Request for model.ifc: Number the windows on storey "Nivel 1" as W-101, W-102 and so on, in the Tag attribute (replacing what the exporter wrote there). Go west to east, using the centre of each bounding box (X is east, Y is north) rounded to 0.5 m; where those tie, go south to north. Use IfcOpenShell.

First a look at what the model holds.

```python
import ifcopenshell
import ifcopenshell.util.element
import ifcopenshell.util.placement

model = ifcopenshell.open("model.ifc")
print(model.schema)
storey = next(s for s in model.by_type("IfcBuildingStorey") if s.Name == "Nivel 1")
windows = [e for e in ifcopenshell.util.element.get_decomposition(storey) if e.is_a("IfcWindow")]
for e in sorted(windows, key=lambda e: e.id()):
    origin = ifcopenshell.util.placement.get_local_placement(e.ObjectPlacement)[:3, 3]
    print(e.id(), e.Tag, e.Name, origin.round(2) + 0.0, sep=" | ")
```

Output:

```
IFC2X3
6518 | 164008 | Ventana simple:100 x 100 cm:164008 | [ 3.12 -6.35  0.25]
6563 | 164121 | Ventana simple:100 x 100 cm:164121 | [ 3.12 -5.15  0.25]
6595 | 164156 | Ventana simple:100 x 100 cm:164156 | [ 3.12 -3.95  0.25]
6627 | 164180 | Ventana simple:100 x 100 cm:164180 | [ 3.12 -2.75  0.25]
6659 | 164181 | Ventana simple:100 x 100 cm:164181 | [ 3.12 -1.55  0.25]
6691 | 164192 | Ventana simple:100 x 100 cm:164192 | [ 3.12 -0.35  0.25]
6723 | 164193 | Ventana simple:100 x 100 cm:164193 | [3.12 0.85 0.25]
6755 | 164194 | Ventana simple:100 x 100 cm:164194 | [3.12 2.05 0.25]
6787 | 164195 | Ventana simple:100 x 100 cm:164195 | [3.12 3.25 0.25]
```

```python
import ifcopenshell
import ifcopenshell.geom
import ifcopenshell.util.element
import ifcopenshell.util.shape

model = ifcopenshell.open("model.ifc")
settings = ifcopenshell.geom.settings()
settings.set("use-world-coords", True)


def centre(element):
    shape = ifcopenshell.geom.create_shape(settings, element)
    return ifcopenshell.util.shape.get_bbox_centroid(shape.geometry)


storey = next(s for s in model.by_type("IfcBuildingStorey") if s.Name == "Nivel 1")
windows = [e for e in ifcopenshell.util.element.get_decomposition(storey) if e.is_a("IfcWindow")]

# Insertion points can sit at a corner or the storey origin, so sort by the geometry (in metres).
centres = {e: centre(e) for e in windows}
windows.sort(key=lambda e: (round(centres[e][0] / 0.5), centres[e][1]))

for i, e in enumerate(windows, start=1):
    number = f"W-1{i:02d}"
    e.Tag = number
    print(e.id(), number)

model.write("model_v2.ifc")
```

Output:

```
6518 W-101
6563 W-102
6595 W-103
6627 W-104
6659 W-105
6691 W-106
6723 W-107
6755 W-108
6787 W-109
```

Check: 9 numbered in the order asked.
